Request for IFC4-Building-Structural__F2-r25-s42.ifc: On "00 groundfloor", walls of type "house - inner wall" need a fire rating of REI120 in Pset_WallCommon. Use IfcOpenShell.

First a look at what the model holds.

```python
import ifcopenshell
import ifcopenshell.util.element

model = ifcopenshell.open("IFC4-Building-Structural__F2-r25-s42.ifc")
print(model.schema)
storey = next(s for s in model.by_type("IfcBuildingStorey") if s.Name == "00 groundfloor")
walls = [e for e in ifcopenshell.util.element.get_decomposition(storey) if e.is_a("IfcWall")]
seen = {}
for e in walls:
    element_type = ifcopenshell.util.element.get_type(e)
    key = (element_type.Name if element_type != e and element_type else None, ifcopenshell.util.element.get_pset(e, "Pset_WallCommon", "FireRating"))
    seen[key] = seen.get(key, 0) + 1
for (name, value), count in sorted(seen.items(), key=str):
    print(count, "x", name, "|", value)
```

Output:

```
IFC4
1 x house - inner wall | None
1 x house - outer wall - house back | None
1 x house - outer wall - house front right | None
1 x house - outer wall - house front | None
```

```python
import ifcopenshell
import ifcopenshell.api.pset
import ifcopenshell.util.element

model = ifcopenshell.open("IFC4-Building-Structural__F2-r25-s42.ifc")

storey = next(s for s in model.by_type("IfcBuildingStorey") if s.Name == "00 groundfloor")
walls = [e for e in ifcopenshell.util.element.get_decomposition(storey) if e.is_a("IfcWall")]

count = 0
for e in walls:
    element_type = ifcopenshell.util.element.get_type(e)
    if element_type in (None, e) or element_type.Name != "house - inner wall":
        continue
    # add_pset returns the element's existing set when there is one.
    pset = ifcopenshell.api.pset.add_pset(model, product=e, name="Pset_WallCommon")
    ifcopenshell.api.pset.edit_pset(model, pset=pset, properties={"FireRating": "REI120"})
    count += 1

print(count, "walls updated")

model.write("IFC4-Building-Structural__F2-r25-s42_updated.ifc")
```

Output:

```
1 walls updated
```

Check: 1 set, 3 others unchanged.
